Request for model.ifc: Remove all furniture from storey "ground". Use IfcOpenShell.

First a look at what the model holds.

```python
import ifcopenshell
import ifcopenshell.util.element

model = ifcopenshell.open("model.ifc")
print(model.schema)
storey = next(s for s in model.by_type("IfcBuildingStorey") if s.Name == "ground")
furniture = [e for e in ifcopenshell.util.element.get_decomposition(storey) if e.is_a("IfcFurnishingElement")]
seen = {}
for e in furniture:
    element_type = ifcopenshell.util.element.get_type(e)
    name = element_type.Name if element_type not in (None, e) else None
    seen[name] = seen.get(name, 0) + 1
for name, count in sorted(seen.items(), key=str):
    print(count, "x", name)
```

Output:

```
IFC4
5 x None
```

```python
import ifcopenshell
import ifcopenshell.api.root
import ifcopenshell.util.element

model = ifcopenshell.open("model.ifc")

storey = next(s for s in model.by_type("IfcBuildingStorey") if s.Name == "ground")
furniture = [e for e in ifcopenshell.util.element.get_decomposition(storey) if e.is_a("IfcFurnishingElement")]

for e in furniture:
    ifcopenshell.api.root.remove_product(model, product=e)
print(len(furniture), "removed")

model.write("model_rev.ifc")
```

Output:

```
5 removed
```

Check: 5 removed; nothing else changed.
